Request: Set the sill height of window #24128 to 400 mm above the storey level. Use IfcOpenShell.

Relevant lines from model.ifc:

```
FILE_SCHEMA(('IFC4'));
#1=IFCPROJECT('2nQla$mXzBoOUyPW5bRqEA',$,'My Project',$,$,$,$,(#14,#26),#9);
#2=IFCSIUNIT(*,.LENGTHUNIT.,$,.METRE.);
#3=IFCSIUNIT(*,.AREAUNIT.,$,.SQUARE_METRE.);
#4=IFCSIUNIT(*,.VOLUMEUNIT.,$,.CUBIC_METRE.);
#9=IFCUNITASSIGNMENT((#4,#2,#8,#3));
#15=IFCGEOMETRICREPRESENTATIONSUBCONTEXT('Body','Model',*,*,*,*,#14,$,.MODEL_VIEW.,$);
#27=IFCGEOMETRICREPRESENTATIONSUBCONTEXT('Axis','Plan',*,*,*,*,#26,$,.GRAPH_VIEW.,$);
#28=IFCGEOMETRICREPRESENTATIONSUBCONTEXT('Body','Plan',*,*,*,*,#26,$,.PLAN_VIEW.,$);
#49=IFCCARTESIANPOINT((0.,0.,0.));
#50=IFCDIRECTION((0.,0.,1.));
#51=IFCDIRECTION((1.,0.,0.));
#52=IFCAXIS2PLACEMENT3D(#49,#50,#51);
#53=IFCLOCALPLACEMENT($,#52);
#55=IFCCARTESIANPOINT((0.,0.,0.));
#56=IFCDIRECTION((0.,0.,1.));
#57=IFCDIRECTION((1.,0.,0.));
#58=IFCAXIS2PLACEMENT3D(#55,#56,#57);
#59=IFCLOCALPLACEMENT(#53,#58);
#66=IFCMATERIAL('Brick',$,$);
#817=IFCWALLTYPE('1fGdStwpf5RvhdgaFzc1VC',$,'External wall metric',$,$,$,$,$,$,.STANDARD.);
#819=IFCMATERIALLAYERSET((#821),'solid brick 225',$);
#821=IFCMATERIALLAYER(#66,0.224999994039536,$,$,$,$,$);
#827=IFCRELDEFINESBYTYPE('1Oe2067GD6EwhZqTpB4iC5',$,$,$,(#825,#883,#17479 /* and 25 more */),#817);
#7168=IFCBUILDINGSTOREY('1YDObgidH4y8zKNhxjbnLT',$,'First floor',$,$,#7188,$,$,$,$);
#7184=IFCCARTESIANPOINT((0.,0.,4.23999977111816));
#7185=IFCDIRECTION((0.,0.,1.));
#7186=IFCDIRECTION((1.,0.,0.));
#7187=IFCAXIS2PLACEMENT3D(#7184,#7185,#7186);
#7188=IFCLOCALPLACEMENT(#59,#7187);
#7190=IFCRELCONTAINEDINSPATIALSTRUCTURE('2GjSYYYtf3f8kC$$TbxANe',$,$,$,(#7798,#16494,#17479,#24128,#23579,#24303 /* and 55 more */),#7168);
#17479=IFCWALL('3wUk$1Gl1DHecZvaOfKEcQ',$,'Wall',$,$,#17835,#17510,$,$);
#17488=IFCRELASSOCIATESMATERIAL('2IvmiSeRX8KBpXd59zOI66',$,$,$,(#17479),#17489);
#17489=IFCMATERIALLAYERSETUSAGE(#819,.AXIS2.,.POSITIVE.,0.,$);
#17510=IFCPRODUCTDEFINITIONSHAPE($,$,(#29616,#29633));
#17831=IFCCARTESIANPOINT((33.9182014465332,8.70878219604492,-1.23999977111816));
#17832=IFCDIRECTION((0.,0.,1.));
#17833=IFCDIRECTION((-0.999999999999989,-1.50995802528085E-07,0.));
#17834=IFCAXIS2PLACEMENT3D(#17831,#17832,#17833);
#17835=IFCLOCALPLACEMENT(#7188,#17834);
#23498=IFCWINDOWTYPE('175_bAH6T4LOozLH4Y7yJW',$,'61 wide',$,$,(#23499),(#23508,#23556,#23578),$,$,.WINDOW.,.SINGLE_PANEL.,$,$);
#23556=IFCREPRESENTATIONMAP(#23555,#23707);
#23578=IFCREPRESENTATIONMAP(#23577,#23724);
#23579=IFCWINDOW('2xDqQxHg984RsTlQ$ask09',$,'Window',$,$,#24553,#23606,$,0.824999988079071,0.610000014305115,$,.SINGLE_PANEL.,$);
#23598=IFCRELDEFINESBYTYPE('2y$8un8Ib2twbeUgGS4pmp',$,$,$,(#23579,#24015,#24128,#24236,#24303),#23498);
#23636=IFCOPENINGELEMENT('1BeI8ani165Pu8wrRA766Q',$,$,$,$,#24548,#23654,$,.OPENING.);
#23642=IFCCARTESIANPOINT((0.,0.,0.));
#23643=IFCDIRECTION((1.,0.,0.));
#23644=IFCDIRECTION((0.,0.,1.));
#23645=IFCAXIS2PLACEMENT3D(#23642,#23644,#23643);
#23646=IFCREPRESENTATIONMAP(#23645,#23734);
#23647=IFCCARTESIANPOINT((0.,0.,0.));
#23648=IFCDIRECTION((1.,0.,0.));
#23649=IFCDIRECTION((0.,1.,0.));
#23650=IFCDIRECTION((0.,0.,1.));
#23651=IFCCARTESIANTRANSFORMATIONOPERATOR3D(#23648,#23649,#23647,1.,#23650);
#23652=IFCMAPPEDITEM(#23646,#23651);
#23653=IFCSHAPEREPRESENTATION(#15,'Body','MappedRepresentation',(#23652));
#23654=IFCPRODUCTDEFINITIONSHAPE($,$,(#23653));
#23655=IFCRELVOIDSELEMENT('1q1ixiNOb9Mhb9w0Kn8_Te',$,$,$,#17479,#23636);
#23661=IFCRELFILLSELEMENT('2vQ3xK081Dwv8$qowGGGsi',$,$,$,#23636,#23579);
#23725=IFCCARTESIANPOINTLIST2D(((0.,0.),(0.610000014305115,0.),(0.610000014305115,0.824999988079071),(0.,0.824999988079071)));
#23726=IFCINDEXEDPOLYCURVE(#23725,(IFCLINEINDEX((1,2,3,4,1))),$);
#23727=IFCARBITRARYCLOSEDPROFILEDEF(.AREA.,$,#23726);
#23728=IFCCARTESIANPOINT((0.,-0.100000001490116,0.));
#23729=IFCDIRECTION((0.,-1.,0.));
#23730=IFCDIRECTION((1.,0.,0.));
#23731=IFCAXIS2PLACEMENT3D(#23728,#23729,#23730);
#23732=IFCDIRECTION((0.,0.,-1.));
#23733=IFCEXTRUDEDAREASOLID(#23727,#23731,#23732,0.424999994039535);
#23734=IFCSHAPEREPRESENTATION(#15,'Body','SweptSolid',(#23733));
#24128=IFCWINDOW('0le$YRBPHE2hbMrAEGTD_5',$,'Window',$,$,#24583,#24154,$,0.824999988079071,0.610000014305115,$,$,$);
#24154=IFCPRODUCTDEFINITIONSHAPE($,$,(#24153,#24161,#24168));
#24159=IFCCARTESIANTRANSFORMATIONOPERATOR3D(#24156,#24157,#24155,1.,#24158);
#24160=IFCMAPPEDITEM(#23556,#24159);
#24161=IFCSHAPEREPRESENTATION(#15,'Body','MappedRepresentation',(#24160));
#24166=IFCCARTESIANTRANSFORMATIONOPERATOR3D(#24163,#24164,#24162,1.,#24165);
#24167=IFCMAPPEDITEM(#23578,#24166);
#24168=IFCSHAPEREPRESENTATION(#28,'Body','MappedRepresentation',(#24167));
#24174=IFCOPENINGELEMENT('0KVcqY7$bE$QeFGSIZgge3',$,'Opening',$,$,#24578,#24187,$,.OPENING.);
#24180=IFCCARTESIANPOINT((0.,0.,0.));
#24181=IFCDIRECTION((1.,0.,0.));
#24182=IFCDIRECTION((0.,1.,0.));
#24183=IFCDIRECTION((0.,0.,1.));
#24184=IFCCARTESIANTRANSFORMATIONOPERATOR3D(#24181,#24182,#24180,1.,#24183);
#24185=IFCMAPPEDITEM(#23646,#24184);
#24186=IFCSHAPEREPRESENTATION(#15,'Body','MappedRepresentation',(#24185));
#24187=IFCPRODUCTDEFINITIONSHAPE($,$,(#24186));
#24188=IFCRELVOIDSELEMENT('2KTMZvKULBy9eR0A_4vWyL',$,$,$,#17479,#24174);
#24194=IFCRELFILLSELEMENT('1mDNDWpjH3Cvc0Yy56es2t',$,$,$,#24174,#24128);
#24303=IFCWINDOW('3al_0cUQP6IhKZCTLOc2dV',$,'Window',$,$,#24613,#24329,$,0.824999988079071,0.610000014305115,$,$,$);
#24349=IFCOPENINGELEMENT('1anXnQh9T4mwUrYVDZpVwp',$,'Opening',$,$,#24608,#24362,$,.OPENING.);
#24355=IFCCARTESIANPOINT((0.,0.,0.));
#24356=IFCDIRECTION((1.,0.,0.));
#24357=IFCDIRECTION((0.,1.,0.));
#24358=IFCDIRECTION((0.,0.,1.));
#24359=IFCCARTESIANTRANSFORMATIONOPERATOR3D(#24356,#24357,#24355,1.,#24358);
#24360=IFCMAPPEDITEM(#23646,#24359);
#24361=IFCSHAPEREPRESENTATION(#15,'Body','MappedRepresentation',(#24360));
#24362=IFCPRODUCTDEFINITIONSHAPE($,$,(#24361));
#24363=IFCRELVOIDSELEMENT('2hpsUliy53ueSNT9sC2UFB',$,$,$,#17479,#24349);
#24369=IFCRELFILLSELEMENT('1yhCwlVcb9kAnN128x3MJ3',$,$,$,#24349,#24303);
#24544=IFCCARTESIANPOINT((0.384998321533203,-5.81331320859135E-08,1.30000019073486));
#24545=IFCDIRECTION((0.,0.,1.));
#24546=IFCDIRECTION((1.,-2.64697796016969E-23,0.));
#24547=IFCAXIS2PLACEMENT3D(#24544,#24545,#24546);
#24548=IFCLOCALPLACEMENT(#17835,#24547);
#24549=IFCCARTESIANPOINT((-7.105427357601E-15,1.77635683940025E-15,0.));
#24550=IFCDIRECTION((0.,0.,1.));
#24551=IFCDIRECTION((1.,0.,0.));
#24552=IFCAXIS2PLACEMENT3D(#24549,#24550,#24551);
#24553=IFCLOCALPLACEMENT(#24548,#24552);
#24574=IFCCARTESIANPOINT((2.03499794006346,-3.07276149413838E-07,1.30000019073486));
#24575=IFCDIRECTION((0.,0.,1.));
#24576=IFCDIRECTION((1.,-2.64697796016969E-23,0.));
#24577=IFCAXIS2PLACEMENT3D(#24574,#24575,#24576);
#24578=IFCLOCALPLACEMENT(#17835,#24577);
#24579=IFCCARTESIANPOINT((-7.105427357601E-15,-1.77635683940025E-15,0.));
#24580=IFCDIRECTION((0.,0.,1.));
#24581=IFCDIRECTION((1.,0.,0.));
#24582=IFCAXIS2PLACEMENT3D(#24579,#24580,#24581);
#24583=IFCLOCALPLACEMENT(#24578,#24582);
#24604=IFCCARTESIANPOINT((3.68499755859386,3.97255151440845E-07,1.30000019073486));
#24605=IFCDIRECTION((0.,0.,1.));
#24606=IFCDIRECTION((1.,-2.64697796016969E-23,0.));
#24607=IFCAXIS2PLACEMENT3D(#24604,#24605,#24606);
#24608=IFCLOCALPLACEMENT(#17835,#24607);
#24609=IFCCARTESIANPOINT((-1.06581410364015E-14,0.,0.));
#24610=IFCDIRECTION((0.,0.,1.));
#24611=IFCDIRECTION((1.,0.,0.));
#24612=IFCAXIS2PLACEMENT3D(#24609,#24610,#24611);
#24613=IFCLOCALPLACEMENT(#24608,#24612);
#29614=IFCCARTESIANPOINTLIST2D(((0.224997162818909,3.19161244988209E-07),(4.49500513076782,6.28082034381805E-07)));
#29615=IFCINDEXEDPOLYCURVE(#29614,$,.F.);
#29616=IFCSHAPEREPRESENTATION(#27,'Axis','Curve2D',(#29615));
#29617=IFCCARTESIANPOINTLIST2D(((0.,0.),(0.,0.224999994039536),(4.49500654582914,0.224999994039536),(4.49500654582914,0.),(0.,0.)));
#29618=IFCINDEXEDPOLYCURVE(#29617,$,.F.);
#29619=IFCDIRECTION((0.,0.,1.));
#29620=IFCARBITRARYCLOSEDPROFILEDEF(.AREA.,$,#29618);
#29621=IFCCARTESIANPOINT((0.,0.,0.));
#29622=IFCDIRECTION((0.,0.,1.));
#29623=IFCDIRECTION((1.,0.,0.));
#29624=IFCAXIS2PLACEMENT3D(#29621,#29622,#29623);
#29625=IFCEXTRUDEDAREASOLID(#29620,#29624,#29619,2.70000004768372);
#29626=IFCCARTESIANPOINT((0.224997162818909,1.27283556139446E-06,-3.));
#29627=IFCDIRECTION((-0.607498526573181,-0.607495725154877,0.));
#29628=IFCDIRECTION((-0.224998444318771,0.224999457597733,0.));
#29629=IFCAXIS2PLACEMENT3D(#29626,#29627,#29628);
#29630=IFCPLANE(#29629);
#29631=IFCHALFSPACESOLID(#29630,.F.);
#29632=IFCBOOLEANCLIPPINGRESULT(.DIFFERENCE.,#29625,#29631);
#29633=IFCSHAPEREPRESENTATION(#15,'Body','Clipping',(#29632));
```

```python
import numpy as np
import ifcopenshell
import ifcopenshell.api.geometry
import ifcopenshell.geom
import ifcopenshell.util.element
import ifcopenshell.util.placement
import ifcopenshell.util.shape
import ifcopenshell.util.unit

model = ifcopenshell.open("model.ifc")
unit_scale = ifcopenshell.util.unit.calculate_unit_scale(model)

window = model.by_guid("0le$YRBPHE2hbMrAEGTD_5")
opening = window.FillsVoids[0].RelatingOpeningElement
storey = ifcopenshell.util.element.get_container(window, ifc_class="IfcBuildingStorey")
level = ifcopenshell.util.placement.get_local_placement(storey.ObjectPlacement)[2, 3]

# The opening's origin need not be at the sill, so measure its lowest point.
shape = ifcopenshell.geom.create_shape(ifcopenshell.geom.settings(), opening)
bottom = ifcopenshell.util.shape.get_shape_bottom_elevation(shape, shape.geometry) / unit_scale
dz = level + 0.4 / unit_scale - bottom

shift = np.array([0.0, 0.0, dz])
# The window is placed relative to its opening, so it follows when the opening moves.
matrix = ifcopenshell.util.placement.get_local_placement(opening.ObjectPlacement)
matrix[:3, 3] += shift
ifcopenshell.api.geometry.edit_object_placement(
    model, product=opening, matrix=matrix, is_si=False, should_transform_children=True
)

print(f"moved by {dz * unit_scale:+.3f} m")

model.write("model_rev.ifc")
```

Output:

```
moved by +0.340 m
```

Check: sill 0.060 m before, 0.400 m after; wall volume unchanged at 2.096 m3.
